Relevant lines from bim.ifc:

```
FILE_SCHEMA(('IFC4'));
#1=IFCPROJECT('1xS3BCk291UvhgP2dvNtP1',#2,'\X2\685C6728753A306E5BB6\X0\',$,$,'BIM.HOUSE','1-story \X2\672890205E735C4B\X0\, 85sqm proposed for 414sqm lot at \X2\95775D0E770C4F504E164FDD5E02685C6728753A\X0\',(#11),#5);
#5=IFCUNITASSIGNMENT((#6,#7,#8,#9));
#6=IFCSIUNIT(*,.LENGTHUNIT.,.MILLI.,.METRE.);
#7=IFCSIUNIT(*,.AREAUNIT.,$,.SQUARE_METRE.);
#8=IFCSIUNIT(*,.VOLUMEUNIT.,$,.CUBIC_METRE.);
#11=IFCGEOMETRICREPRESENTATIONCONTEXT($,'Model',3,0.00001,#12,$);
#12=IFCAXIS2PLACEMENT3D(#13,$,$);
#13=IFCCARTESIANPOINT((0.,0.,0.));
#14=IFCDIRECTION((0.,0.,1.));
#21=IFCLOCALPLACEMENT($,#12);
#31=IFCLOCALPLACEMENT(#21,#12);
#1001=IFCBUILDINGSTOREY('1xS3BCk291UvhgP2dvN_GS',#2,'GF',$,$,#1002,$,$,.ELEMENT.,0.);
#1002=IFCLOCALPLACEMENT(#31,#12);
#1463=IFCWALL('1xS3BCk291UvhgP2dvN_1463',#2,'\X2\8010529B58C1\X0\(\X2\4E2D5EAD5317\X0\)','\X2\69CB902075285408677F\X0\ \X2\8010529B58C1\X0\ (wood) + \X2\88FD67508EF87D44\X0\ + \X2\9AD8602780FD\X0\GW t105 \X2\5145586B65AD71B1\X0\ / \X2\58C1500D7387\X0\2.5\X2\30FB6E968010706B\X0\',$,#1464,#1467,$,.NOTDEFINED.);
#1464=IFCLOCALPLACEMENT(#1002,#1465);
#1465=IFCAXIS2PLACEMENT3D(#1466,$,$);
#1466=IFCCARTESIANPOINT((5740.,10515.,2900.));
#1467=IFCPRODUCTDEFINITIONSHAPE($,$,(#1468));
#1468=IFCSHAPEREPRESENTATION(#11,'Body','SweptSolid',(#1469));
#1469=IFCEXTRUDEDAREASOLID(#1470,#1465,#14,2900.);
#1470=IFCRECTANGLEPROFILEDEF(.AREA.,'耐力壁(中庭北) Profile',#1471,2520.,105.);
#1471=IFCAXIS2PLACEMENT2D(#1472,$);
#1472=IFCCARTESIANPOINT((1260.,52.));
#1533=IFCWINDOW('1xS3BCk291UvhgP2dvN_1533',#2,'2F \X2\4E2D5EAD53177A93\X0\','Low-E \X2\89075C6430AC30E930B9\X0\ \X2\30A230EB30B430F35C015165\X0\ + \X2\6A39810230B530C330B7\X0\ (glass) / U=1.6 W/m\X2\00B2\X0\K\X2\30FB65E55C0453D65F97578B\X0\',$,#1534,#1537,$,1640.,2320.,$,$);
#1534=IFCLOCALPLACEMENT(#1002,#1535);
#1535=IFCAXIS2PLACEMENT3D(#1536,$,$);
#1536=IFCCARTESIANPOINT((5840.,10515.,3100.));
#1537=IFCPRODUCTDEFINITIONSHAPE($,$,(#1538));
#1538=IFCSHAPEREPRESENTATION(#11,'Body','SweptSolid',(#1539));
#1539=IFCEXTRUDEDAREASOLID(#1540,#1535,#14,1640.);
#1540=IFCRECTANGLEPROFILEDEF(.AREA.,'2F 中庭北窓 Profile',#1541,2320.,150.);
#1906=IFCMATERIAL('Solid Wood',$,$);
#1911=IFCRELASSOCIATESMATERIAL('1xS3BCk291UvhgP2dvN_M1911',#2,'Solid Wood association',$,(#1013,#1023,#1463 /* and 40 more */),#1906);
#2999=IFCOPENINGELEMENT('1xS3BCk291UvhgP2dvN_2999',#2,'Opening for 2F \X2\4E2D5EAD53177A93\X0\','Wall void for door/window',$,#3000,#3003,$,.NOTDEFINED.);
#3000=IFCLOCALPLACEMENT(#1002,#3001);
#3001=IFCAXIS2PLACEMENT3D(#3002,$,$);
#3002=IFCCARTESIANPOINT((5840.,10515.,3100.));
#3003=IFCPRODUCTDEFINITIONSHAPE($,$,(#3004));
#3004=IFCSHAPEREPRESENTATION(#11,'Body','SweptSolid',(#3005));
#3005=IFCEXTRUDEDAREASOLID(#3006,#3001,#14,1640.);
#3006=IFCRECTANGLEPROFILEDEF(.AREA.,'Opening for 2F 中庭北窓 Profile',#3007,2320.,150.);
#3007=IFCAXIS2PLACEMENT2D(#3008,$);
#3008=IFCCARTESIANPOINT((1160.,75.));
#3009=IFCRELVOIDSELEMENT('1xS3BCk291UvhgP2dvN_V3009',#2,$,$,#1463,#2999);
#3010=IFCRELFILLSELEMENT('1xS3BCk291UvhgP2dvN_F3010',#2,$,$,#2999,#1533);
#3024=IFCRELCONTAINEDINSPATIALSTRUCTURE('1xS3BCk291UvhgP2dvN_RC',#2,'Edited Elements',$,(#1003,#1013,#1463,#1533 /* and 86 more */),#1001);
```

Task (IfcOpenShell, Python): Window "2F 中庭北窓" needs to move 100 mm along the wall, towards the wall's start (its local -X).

```python
import ifcopenshell
import ifcopenshell.api.geometry
import ifcopenshell.util.placement

model = ifcopenshell.open("bim.ifc")

window = model.by_guid("1xS3BCk291UvhgP2dvN_1533")
opening = window.FillsVoids[0].RelatingOpeningElement
wall = opening.VoidsElements[0].RelatingBuildingElement

wall_matrix = ifcopenshell.util.placement.get_local_placement(wall.ObjectPlacement)
shift = wall_matrix[:3, 0] * -100.0
before = ifcopenshell.util.placement.get_local_placement(window.ObjectPlacement)[:3, 3].copy()

# The window is not placed relative to its opening, so move both.
for product in (opening, window):
    matrix = ifcopenshell.util.placement.get_local_placement(product.ObjectPlacement)
    matrix[:3, 3] += shift
    ifcopenshell.api.geometry.edit_object_placement(model, product=product, matrix=matrix, is_si=False)

after = ifcopenshell.util.placement.get_local_placement(window.ObjectPlacement)[:3, 3]
print("window moved by", (after - before).round(3) + 0.0)

model.write("bim_updated.ifc")
```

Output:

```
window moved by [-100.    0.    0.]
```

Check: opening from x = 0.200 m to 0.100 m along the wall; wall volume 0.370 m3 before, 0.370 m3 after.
